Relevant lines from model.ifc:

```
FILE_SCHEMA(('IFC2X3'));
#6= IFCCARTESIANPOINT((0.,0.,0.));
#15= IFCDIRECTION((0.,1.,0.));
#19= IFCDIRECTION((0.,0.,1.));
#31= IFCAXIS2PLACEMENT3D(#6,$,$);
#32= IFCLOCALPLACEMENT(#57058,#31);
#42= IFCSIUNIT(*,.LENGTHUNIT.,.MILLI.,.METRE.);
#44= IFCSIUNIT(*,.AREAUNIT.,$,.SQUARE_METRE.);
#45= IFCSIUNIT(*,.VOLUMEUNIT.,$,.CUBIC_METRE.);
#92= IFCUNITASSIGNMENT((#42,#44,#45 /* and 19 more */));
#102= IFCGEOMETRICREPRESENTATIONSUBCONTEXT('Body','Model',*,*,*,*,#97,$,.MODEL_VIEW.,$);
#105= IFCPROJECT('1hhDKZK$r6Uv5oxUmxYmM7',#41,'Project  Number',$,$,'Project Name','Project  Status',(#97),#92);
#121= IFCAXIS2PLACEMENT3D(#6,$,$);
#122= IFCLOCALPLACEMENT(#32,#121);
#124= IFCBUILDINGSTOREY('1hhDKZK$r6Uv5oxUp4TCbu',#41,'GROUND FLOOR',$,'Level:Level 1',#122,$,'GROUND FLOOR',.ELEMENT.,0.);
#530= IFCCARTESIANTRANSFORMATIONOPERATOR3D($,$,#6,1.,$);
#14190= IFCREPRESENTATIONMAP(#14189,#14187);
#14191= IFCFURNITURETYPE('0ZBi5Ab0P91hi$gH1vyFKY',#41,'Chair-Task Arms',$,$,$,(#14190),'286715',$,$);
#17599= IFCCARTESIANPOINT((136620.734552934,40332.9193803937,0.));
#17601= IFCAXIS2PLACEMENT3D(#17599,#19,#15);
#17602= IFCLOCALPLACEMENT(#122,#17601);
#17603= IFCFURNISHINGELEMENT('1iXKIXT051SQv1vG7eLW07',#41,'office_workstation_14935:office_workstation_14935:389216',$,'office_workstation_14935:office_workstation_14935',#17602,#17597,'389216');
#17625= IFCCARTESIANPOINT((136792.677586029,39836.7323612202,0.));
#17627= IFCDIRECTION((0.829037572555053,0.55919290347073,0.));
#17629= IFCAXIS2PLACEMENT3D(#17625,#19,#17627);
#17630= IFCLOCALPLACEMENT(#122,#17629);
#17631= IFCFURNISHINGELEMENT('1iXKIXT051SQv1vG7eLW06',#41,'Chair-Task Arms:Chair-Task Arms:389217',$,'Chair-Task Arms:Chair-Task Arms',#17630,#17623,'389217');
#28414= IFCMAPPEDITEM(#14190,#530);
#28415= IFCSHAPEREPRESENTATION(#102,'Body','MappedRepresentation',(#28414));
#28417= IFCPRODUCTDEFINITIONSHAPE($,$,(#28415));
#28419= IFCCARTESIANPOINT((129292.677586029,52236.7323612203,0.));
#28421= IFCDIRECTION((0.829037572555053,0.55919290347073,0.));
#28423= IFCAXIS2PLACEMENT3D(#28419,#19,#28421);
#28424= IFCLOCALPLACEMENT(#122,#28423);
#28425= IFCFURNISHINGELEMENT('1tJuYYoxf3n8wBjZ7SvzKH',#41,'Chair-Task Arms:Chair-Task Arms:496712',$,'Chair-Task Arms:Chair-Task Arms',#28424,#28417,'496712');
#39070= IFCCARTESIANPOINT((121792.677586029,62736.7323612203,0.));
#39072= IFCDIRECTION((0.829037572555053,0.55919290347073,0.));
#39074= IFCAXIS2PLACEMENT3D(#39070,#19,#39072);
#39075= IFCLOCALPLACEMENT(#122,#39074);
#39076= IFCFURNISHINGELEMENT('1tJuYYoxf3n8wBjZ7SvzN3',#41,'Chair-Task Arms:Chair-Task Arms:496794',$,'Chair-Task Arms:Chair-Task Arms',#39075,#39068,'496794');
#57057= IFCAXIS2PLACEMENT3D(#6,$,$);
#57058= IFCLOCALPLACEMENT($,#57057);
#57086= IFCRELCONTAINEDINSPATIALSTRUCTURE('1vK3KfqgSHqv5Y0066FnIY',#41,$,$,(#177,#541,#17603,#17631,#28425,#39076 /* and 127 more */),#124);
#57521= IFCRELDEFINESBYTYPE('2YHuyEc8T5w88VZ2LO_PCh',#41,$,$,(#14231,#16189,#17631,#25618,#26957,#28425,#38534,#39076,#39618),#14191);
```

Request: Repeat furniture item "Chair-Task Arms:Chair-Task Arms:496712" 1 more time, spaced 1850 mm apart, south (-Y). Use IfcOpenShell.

```python
import numpy as np
import ifcopenshell
import ifcopenshell.api.geometry
import ifcopenshell.api.root
import ifcopenshell.util.element
import ifcopenshell.util.placement
import ifcopenshell.util.unit

model = ifcopenshell.open("model.ifc")
unit_scale = ifcopenshell.util.unit.calculate_unit_scale(model)


def reuse_history(source, copy):
    """copy_class also copies each property set's owner history, people and application; keep the originals."""
    for rel in copy.IsDefinedBy:
        if rel.is_a("IfcRelDefinesByProperties") and (history := rel.RelatingPropertyDefinition.OwnerHistory):
            rel.RelatingPropertyDefinition.OwnerHistory = source.OwnerHistory
            ifcopenshell.util.element.remove_deep2(model, history)


source = model.by_guid("1tJuYYoxf3n8wBjZ7SvzKH")
base = ifcopenshell.util.placement.get_local_placement(source.ObjectPlacement)
step = np.array([0.0, -1.0, 0.0]) * 1.85 / unit_scale

for i in range(1, 2):
    copy = ifcopenshell.api.root.copy_class(model, product=source)
    copy.Representation = ifcopenshell.util.element.copy_deep(
        model, source.Representation, exclude=["IfcGeometricRepresentationContext", "IfcRepresentationMap"]
    )
    copy.Name = "Chair-Task Arms:Chair-Task Arms"
    copy.Tag = None
    reuse_history(source, copy)
    matrix = base.copy()
    matrix[:3, 3] += i * step
    print("added at", matrix[:3, 3].round(3) + 0.0)
    ifcopenshell.api.geometry.edit_object_placement(model, product=copy, matrix=matrix, is_si=False)

model.write("model-out.ifc")
```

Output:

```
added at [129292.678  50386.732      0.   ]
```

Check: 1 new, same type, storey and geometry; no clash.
